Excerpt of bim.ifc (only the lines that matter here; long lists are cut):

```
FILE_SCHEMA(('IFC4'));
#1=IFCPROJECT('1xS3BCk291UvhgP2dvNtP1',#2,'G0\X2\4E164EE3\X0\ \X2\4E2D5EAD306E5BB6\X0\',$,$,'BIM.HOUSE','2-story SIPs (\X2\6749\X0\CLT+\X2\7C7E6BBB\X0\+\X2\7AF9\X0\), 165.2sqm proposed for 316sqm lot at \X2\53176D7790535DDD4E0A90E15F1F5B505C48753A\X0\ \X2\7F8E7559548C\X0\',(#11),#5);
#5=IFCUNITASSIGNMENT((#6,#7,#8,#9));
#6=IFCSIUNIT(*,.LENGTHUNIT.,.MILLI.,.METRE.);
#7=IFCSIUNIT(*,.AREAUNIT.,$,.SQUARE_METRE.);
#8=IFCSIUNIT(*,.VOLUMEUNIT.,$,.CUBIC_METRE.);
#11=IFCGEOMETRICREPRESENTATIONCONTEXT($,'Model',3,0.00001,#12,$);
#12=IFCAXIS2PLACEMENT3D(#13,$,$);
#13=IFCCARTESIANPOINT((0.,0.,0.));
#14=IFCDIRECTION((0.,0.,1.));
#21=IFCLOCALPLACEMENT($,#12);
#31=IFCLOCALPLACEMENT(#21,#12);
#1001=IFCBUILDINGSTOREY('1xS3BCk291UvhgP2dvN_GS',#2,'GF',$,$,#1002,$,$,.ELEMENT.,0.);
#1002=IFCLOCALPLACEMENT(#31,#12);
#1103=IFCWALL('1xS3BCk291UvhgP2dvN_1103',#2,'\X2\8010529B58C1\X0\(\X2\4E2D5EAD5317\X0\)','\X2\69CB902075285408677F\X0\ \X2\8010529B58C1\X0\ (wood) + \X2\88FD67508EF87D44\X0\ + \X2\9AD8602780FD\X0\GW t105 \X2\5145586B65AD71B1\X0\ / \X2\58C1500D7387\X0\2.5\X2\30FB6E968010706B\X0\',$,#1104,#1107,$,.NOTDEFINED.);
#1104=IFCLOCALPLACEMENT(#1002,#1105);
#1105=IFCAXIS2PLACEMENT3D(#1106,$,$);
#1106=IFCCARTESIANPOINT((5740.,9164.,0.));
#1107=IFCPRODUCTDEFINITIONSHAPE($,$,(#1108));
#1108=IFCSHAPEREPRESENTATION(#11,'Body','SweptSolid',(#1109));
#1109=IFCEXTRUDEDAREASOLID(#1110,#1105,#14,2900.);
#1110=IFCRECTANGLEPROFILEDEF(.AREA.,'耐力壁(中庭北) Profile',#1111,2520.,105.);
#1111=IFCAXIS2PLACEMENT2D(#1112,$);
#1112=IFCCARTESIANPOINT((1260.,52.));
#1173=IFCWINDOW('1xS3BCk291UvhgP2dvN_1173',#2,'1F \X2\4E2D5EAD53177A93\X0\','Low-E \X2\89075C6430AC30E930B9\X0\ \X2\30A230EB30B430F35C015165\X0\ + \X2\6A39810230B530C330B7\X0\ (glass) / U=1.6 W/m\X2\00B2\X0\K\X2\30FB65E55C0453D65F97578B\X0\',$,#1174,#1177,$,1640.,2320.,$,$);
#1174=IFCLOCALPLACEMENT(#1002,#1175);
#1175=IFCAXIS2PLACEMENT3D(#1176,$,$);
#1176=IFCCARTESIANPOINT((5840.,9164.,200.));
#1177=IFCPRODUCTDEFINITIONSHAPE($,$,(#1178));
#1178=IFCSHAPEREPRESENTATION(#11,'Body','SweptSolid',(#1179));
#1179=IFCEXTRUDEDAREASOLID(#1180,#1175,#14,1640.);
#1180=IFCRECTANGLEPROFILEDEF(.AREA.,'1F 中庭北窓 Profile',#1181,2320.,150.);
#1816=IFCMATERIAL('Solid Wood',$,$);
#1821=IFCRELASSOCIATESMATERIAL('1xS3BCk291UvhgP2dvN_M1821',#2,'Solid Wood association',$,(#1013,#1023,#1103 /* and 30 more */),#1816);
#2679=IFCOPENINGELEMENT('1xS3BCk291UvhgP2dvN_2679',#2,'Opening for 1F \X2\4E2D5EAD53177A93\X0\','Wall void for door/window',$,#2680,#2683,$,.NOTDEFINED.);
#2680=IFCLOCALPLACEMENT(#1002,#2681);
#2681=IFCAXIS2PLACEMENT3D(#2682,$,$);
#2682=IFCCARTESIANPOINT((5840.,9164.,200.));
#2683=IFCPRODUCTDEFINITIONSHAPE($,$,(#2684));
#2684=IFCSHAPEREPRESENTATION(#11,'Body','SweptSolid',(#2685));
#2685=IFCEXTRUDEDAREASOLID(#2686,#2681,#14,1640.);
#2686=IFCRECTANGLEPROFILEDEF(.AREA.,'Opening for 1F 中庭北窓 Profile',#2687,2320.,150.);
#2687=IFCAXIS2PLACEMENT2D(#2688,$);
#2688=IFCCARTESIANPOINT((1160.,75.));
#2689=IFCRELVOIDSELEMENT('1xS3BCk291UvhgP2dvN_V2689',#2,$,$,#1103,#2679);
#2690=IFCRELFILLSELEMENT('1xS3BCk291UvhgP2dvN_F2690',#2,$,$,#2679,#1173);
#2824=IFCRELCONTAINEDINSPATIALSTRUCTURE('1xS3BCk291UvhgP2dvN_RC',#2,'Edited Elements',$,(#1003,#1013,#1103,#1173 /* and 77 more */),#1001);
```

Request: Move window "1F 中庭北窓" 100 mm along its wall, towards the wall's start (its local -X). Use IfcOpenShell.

```python
import ifcopenshell
import ifcopenshell.api.geometry
import ifcopenshell.util.placement
import ifcopenshell.util.unit

model = ifcopenshell.open("bim.ifc")
unit_scale = ifcopenshell.util.unit.calculate_unit_scale(model)

window = model.by_id(1173)
opening = window.FillsVoids[0].RelatingOpeningElement
wall = opening.VoidsElements[0].RelatingBuildingElement

wall_matrix = ifcopenshell.util.placement.get_local_placement(wall.ObjectPlacement)
shift = wall_matrix[:3, 0] * -0.1 / unit_scale
before = ifcopenshell.util.placement.get_local_placement(window.ObjectPlacement)[:3, 3].copy()

# The window is not placed relative to its opening, so move both.
for product in (opening, window):
    matrix = ifcopenshell.util.placement.get_local_placement(product.ObjectPlacement)
    matrix[:3, 3] += shift
    ifcopenshell.api.geometry.edit_object_placement(model, product=product, matrix=matrix, is_si=False)

after = ifcopenshell.util.placement.get_local_placement(window.ObjectPlacement)[:3, 3]
print("window moved by", (after - before).round(3) + 0.0)

model.write("bim_rev.ifc")
```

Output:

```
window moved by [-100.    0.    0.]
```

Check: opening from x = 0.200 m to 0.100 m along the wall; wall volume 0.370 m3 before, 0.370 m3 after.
